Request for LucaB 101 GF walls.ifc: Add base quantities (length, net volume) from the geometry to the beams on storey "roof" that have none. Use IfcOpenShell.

First a look at what the model holds.

```python
import ifcopenshell
import ifcopenshell.util.element
import ifcopenshell.util.unit

model = ifcopenshell.open("LucaB 101 GF walls.ifc")
print(model.schema)
for unit_type in ("LENGTHUNIT", "AREAUNIT", "VOLUMEUNIT"):
    print(unit_type, ifcopenshell.util.unit.calculate_unit_scale(model, unit_type))
storey = next(s for s in model.by_type("IfcBuildingStorey") if s.Name == "roof")
beams = [e for e in ifcopenshell.util.element.get_decomposition(storey) if e.is_a("IfcBeam")]
for e in sorted(beams, key=lambda e: e.id()):
    print(e.id(), e.is_a(), e.Name, list(ifcopenshell.util.element.get_psets(e, qtos_only=True)), sep=" | ")
```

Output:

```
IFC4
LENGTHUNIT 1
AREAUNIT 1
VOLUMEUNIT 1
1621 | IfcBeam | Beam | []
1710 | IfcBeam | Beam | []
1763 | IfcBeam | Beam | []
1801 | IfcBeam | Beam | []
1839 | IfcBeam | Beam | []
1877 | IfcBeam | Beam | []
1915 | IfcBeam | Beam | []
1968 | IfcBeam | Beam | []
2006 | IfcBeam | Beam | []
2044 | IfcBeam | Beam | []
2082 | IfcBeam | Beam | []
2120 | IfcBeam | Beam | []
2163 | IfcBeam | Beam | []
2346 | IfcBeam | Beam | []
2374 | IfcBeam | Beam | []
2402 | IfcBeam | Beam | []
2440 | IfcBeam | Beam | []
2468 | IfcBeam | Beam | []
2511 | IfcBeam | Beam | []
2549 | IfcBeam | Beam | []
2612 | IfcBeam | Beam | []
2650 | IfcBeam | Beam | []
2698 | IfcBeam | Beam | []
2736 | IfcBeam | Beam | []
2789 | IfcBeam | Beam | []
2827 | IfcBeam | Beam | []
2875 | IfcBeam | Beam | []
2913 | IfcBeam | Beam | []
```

```python
import ifcopenshell
import ifcopenshell.api.pset
import ifcopenshell.geom
import ifcopenshell.util.element
import ifcopenshell.util.shape
import ifcopenshell.util.unit

model = ifcopenshell.open("LucaB 101 GF walls.ifc")
unit_scale = ifcopenshell.util.unit.calculate_unit_scale(model)
volume_scale = ifcopenshell.util.unit.calculate_unit_scale(model, "VOLUMEUNIT")
settings = ifcopenshell.geom.settings()

storey = next(s for s in model.by_type("IfcBuildingStorey") if s.Name == "roof")
beams = [e for e in ifcopenshell.util.element.get_decomposition(storey) if e.is_a("IfcBeam")]

for e in sorted(beams, key=lambda e: e.id()):
    if ifcopenshell.util.element.get_psets(e, qtos_only=True, should_inherit=False):
        continue
    # Geometry comes back in metres, in the element's own axes.
    shape = ifcopenshell.geom.create_shape(settings, e)
    values = {
        "Length": ifcopenshell.util.shape.get_max_xyz(shape.geometry) / unit_scale,
        "NetVolume": ifcopenshell.util.shape.get_volume(shape.geometry) / volume_scale,
    }
    qto = ifcopenshell.api.pset.add_qto(model, product=e, name="Qto_BeamBaseQuantities")
    ifcopenshell.api.pset.edit_qto(model, qto=qto, properties=values)
    print(e.id(), {k: round(v, 3) for k, v in values.items()})

model.write("LucaB 101 GF walls-out.ifc")
```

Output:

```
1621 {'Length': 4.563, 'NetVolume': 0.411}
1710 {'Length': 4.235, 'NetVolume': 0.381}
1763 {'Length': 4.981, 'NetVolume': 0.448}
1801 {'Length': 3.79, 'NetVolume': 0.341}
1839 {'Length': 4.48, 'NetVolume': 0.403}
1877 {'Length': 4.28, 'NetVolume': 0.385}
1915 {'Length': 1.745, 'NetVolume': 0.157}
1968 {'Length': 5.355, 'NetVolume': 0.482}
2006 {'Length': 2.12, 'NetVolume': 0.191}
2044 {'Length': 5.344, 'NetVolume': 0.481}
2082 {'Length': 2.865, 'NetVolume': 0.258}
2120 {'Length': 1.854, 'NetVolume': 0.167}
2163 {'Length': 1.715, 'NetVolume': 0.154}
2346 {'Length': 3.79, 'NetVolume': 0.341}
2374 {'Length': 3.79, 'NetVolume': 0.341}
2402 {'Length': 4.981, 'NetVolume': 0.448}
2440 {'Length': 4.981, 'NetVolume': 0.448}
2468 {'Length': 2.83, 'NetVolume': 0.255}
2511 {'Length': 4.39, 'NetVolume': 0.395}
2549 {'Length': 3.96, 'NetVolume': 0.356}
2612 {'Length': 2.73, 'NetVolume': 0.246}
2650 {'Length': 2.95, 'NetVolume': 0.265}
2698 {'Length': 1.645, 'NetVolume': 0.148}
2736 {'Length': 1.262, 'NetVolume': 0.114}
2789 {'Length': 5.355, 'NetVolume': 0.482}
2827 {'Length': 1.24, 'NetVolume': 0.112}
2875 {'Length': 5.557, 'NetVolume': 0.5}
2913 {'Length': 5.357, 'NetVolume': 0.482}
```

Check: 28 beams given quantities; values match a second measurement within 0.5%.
